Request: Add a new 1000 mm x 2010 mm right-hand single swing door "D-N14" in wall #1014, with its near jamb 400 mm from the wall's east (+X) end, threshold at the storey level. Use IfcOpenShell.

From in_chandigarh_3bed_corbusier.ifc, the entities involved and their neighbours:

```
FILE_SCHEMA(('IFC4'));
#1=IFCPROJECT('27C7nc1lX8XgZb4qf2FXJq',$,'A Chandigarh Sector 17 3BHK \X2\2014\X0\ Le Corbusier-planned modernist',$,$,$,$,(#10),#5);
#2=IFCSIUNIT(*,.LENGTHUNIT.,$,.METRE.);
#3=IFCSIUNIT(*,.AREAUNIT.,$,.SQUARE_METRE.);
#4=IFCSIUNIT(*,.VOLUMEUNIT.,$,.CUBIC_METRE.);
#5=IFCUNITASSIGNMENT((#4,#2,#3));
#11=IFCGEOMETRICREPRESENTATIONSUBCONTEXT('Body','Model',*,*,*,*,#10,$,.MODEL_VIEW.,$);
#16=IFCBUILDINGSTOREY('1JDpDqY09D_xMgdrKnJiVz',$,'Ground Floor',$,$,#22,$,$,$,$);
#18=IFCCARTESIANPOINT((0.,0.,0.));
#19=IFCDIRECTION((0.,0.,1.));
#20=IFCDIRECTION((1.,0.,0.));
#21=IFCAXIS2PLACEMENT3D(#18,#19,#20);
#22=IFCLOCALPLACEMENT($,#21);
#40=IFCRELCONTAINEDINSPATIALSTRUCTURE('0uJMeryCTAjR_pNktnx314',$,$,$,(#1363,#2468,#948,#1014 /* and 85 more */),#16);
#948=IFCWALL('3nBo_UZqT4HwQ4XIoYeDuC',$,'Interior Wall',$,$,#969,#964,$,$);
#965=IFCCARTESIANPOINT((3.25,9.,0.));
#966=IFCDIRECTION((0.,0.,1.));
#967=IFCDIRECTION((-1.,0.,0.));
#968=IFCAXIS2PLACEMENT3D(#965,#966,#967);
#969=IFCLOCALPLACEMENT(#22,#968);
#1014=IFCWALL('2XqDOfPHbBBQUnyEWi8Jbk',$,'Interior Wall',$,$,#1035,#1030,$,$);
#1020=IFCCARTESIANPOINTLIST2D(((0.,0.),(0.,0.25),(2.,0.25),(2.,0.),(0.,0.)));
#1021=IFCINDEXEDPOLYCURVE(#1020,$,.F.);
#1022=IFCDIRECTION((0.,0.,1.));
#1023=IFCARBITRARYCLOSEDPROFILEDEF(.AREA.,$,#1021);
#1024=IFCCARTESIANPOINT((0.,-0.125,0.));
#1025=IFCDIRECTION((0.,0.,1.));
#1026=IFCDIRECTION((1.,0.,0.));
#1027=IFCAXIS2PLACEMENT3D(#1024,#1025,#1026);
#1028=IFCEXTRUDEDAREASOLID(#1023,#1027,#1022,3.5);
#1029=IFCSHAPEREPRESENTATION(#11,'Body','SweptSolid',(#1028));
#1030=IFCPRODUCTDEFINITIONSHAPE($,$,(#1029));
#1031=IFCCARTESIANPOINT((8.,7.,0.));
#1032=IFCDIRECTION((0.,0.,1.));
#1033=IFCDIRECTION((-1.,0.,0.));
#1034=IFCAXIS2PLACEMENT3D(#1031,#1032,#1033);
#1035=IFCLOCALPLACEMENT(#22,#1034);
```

```python
import numpy as np
import ifcopenshell
import ifcopenshell.api.feature
import ifcopenshell.api.geometry
import ifcopenshell.api.root
import ifcopenshell.api.spatial
import ifcopenshell.geom
import ifcopenshell.util.element
import ifcopenshell.util.placement
import ifcopenshell.util.representation
import ifcopenshell.util.shape
import ifcopenshell.util.unit

model = ifcopenshell.open("in_chandigarh_3bed_corbusier.ifc")
unit_scale = ifcopenshell.util.unit.calculate_unit_scale(model)
settings = ifcopenshell.geom.settings()


def volume(element):
    """Net volume in cubic metres, openings subtracted."""
    shape = ifcopenshell.geom.create_shape(settings, element)
    return ifcopenshell.util.shape.get_volume(shape.geometry)


wall = model.by_id(1014)
storey = ifcopenshell.util.element.get_container(wall, ifc_class="IfcBuildingStorey")
context = ifcopenshell.util.representation.get_context(model, "Model", "Body", "MODEL_VIEW")
before = volume(wall)

width, height, from_end, sill = 1, 2.01, 0.4, 0.0  # metres

# The wall runs along its own X axis, and the end named is its -X end.
wall_shape = ifcopenshell.geom.create_shape(settings, wall)
x, y, z = ifcopenshell.util.shape.get_vertices(wall_shape.geometry).T
start = x.min() + from_end
face, thickness = float(y.min()), float(y.max() - y.min())
wall_matrix = ifcopenshell.util.placement.get_local_placement(wall.ObjectPlacement)
level = ifcopenshell.util.placement.get_local_placement(storey.ObjectPlacement)[2, 3]


def in_wall(x, y):
    """Placement at x, y metres in the wall's axes, at sill height."""
    matrix = wall_matrix.copy()
    matrix[:, 3] = wall_matrix @ np.array([x / unit_scale, y / unit_scale, 0.0, 1.0])
    matrix[2, 3] = level + sill / unit_scale
    return matrix


# Opening: a box that overshoots both wall faces by 50 mm.
opening = ifcopenshell.api.root.create_entity(model, ifc_class="IfcOpeningElement", predefined_type="OPENING")
box = ifcopenshell.api.geometry.add_wall_representation(
    model, context=context, length=width, height=height, thickness=thickness + 0.1
)
ifcopenshell.api.geometry.assign_representation(model, product=opening, representation=box)
ifcopenshell.api.geometry.edit_object_placement(model, product=opening, matrix=in_wall(start, face - 0.05), is_si=False)
ifcopenshell.api.feature.add_feature(model, feature=opening, element=wall)

door = ifcopenshell.api.root.create_entity(model, ifc_class="IfcDoor", name="D-N14", predefined_type="DOOR")
door.OverallWidth, door.OverallHeight = width / unit_scale, height / unit_scale
door.OperationType = "SINGLE_SWING_RIGHT"
body = ifcopenshell.api.geometry.add_door_representation(
    model,
    context=context,
    overall_width=door.OverallWidth,
    overall_height=door.OverallHeight,
    operation_type="SINGLE_SWING_RIGHT",
    lining_properties={"LiningDepth": thickness / unit_scale, "ThresholdDepth": thickness / unit_scale},
)
ifcopenshell.api.geometry.assign_representation(model, product=door, representation=body)
ifcopenshell.api.spatial.assign_container(model, products=[door], relating_structure=storey)
ifcopenshell.api.feature.add_filling(model, opening=opening, element=door)

# The lining spans the wall, so the door starts at the wall face.
ifcopenshell.api.geometry.edit_object_placement(model, product=door, matrix=in_wall(start, face), is_si=False)

after = volume(wall)

print(f"wall volume {before:.3f} -> {after:.3f} m3")

model.write("in_chandigarh_3bed_corbusier_edited.ifc")
```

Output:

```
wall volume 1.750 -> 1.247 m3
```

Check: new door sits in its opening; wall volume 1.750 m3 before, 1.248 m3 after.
